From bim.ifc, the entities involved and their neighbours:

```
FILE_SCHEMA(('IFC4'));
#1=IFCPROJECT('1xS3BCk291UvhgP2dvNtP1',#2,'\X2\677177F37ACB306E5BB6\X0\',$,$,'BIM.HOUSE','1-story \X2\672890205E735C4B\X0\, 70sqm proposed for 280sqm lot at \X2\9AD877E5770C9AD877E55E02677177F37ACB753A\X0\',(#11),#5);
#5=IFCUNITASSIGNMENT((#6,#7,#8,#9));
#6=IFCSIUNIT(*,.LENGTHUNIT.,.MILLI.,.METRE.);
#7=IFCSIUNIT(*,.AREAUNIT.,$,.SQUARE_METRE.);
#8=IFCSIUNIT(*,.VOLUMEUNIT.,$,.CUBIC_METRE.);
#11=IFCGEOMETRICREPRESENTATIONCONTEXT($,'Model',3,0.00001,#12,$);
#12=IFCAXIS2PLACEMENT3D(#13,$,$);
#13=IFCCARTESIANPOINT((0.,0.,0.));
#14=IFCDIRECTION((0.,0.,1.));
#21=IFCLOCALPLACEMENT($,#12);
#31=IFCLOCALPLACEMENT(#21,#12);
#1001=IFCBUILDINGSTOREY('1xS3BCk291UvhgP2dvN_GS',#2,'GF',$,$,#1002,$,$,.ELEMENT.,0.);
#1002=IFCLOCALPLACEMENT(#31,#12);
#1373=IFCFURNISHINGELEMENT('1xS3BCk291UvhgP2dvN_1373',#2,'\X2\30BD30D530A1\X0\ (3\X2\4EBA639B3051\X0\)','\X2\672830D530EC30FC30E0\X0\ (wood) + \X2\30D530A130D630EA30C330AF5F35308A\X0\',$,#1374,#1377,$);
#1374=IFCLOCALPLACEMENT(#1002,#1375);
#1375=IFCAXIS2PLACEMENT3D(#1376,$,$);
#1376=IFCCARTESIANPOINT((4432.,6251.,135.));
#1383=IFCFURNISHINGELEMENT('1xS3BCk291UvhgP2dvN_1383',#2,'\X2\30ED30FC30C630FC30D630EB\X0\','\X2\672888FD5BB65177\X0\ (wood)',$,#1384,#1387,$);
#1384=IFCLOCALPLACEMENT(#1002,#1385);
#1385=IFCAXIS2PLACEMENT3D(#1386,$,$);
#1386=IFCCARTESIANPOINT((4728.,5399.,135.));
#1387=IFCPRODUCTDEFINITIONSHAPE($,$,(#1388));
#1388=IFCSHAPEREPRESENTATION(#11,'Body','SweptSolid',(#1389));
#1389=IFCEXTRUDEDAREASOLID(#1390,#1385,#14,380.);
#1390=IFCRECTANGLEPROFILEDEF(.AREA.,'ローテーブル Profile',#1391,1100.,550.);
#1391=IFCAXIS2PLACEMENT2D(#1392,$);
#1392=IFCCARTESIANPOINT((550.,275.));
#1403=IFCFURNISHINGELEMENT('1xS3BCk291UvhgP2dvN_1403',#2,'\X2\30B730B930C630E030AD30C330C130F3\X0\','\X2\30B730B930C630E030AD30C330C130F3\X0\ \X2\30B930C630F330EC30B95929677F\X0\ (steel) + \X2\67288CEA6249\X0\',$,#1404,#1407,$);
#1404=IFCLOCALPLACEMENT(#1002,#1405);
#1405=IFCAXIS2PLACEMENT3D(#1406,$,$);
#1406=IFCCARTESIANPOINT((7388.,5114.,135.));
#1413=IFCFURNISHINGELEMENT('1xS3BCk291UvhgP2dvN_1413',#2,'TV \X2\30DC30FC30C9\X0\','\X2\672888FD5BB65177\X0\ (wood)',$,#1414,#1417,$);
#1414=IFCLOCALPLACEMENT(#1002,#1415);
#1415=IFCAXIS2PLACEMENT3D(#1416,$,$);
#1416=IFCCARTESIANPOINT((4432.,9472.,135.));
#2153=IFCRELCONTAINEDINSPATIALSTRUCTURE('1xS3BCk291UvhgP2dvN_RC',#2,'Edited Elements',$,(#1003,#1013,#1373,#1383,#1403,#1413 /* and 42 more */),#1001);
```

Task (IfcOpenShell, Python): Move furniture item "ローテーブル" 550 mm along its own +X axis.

```python
import ifcopenshell
import ifcopenshell.api.geometry
import ifcopenshell.util.placement
import ifcopenshell.util.unit

model = ifcopenshell.open("bim.ifc")
unit_scale = ifcopenshell.util.unit.calculate_unit_scale(model)

item = model.by_guid("1xS3BCk291UvhgP2dvN_1383")
matrix = ifcopenshell.util.placement.get_local_placement(item.ObjectPlacement)
matrix[:3, 3] += matrix[:3, 0] * 0.55 / unit_scale
ifcopenshell.api.geometry.edit_object_placement(model, product=item, matrix=matrix, is_si=False)

print(ifcopenshell.util.placement.get_local_placement(item.ObjectPlacement).round(3) + 0.0)

model.write("bim_rev.ifc")
```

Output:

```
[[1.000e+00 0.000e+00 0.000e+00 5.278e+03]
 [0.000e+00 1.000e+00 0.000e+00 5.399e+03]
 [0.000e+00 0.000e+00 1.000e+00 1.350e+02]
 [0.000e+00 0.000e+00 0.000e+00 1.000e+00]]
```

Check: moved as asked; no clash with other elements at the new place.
